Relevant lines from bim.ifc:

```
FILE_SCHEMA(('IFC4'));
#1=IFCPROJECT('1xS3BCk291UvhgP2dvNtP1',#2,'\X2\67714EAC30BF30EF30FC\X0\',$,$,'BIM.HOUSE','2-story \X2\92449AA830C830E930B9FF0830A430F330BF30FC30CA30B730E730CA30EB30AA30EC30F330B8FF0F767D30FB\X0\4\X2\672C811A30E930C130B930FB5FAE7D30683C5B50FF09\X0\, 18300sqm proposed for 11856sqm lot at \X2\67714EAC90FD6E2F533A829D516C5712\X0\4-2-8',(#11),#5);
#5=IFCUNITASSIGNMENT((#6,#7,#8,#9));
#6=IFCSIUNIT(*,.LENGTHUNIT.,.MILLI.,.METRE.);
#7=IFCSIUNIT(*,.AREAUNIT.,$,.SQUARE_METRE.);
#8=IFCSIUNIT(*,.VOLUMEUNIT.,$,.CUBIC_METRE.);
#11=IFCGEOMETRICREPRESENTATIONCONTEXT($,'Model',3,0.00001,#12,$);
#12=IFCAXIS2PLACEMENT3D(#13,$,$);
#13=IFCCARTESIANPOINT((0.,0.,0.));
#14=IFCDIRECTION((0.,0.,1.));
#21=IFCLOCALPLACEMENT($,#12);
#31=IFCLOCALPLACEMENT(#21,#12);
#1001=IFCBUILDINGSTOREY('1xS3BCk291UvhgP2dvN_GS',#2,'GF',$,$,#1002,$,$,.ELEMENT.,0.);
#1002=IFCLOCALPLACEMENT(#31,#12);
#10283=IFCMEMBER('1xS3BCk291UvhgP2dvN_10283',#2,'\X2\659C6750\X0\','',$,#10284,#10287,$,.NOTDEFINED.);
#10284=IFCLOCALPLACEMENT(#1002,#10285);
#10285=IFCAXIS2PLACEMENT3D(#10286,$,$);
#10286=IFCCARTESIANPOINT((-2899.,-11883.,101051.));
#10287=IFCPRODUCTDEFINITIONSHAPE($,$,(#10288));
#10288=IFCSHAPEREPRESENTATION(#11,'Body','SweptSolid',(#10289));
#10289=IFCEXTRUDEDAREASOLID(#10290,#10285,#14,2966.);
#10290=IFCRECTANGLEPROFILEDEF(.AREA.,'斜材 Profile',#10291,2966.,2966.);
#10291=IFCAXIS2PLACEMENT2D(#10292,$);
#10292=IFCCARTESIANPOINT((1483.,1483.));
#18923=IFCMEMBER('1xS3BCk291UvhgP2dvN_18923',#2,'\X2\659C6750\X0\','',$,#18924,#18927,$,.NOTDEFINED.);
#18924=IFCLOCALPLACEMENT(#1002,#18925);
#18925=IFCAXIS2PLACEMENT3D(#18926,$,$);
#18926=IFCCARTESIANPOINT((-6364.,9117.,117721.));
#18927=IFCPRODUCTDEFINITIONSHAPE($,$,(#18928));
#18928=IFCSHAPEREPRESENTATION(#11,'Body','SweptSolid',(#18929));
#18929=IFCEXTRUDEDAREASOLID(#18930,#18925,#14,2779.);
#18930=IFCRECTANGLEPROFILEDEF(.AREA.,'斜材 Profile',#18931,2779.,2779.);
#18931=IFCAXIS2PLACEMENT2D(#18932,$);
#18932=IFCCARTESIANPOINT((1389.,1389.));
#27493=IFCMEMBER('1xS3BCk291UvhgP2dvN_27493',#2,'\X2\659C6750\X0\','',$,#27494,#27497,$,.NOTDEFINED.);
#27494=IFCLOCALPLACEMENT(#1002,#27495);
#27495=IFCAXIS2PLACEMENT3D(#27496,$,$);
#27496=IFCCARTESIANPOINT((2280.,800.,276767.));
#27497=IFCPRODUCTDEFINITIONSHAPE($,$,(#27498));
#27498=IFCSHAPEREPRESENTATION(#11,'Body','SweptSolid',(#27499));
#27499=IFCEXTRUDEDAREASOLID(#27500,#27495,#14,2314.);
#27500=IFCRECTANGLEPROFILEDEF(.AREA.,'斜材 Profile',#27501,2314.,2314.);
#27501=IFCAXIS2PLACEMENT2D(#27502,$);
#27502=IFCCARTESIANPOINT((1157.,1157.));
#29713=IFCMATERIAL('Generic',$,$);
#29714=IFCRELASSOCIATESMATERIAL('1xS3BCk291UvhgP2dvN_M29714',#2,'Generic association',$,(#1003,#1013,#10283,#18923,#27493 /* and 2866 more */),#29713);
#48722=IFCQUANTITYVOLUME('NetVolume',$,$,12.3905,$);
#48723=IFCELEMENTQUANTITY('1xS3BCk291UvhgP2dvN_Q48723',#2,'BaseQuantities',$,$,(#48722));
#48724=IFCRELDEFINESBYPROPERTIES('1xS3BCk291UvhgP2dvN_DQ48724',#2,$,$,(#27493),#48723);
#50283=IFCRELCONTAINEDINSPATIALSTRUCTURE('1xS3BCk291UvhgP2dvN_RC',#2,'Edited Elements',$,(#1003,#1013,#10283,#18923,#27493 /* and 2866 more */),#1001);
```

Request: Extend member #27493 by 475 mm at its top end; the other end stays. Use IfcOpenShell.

```python
import ifcopenshell
import ifcopenshell.api.pset
import ifcopenshell.util.element
import ifcopenshell.util.unit

model = ifcopenshell.open("bim.ifc")
unit_scale = ifcopenshell.util.unit.calculate_unit_scale(model)

member = model.by_id(27493)
change = 0.475 / unit_scale

# The extrusion runs towards the end named, so only its depth changes.
body = next(r for r in member.Representation.Representations if r.RepresentationIdentifier == "Body")
solid = body.Items[0]
old_length = solid.Depth
solid.Depth += change

# Update the stored length and volume.
qto = model.by_id(ifcopenshell.util.element.get_pset(member, "BaseQuantities", should_inherit=False)["id"])
ifcopenshell.api.pset.edit_qto(model, qto=qto, properties={
    "NetVolume": ifcopenshell.util.element.get_pset(member, "BaseQuantities", "NetVolume") * solid.Depth / old_length,
})

print(f"length {old_length:g} -> {solid.Depth:g}")

model.write("bim_rev.ifc")
```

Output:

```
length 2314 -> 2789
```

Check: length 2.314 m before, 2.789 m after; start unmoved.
